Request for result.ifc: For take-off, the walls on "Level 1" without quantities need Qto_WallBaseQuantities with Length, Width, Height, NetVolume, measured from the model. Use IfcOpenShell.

First a look at what the model holds.

```python
import ifcopenshell
import ifcopenshell.util.element
import ifcopenshell.util.unit

model = ifcopenshell.open("result.ifc")
print(model.schema)
for unit_type in ("LENGTHUNIT", "AREAUNIT", "VOLUMEUNIT"):
    print(unit_type, ifcopenshell.util.unit.calculate_unit_scale(model, unit_type))
storey = next(s for s in model.by_type("IfcBuildingStorey") if s.Name == "Level 1")
walls = [e for e in ifcopenshell.util.element.get_decomposition(storey) if e.is_a("IfcWall")]
for e in sorted(walls, key=lambda e: e.id()):
    print(e.id(), e.is_a(), e.Name, list(ifcopenshell.util.element.get_psets(e, qtos_only=True)), sep=" | ")
```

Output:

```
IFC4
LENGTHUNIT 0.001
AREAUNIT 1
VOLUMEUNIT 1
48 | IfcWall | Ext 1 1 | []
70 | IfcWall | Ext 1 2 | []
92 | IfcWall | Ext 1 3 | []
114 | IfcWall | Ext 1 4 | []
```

```python
import ifcopenshell
import ifcopenshell.api.pset
import ifcopenshell.geom
import ifcopenshell.util.element
import ifcopenshell.util.shape
import ifcopenshell.util.unit

model = ifcopenshell.open("result.ifc")
unit_scale = ifcopenshell.util.unit.calculate_unit_scale(model)
volume_scale = ifcopenshell.util.unit.calculate_unit_scale(model, "VOLUMEUNIT")
settings = ifcopenshell.geom.settings()

storey = next(s for s in model.by_type("IfcBuildingStorey") if s.Name == "Level 1")
walls = [e for e in ifcopenshell.util.element.get_decomposition(storey) if e.is_a("IfcWall")]

for e in sorted(walls, key=lambda e: e.id()):
    if ifcopenshell.util.element.get_psets(e, qtos_only=True, should_inherit=False):
        continue
    # Geometry comes back in metres, in the element's own axes.
    shape = ifcopenshell.geom.create_shape(settings, e)
    values = {
        "Length": ifcopenshell.util.shape.get_x(shape.geometry) / unit_scale,
        "Width": ifcopenshell.util.shape.get_y(shape.geometry) / unit_scale,
        "Height": ifcopenshell.util.shape.get_z(shape.geometry) / unit_scale,
        "NetVolume": ifcopenshell.util.shape.get_volume(shape.geometry) / volume_scale,
    }
    qto = ifcopenshell.api.pset.add_qto(model, product=e, name="Qto_WallBaseQuantities")
    ifcopenshell.api.pset.edit_qto(model, qto=qto, properties=values)
    print(e.id(), {k: round(v, 3) for k, v in values.items()})

model.write("result-out.ifc")
```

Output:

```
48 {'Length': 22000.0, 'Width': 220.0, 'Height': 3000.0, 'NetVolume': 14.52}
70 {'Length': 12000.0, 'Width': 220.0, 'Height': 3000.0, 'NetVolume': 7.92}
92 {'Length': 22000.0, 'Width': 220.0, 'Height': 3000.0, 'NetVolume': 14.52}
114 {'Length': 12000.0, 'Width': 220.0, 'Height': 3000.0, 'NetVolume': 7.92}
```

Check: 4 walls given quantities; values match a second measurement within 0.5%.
